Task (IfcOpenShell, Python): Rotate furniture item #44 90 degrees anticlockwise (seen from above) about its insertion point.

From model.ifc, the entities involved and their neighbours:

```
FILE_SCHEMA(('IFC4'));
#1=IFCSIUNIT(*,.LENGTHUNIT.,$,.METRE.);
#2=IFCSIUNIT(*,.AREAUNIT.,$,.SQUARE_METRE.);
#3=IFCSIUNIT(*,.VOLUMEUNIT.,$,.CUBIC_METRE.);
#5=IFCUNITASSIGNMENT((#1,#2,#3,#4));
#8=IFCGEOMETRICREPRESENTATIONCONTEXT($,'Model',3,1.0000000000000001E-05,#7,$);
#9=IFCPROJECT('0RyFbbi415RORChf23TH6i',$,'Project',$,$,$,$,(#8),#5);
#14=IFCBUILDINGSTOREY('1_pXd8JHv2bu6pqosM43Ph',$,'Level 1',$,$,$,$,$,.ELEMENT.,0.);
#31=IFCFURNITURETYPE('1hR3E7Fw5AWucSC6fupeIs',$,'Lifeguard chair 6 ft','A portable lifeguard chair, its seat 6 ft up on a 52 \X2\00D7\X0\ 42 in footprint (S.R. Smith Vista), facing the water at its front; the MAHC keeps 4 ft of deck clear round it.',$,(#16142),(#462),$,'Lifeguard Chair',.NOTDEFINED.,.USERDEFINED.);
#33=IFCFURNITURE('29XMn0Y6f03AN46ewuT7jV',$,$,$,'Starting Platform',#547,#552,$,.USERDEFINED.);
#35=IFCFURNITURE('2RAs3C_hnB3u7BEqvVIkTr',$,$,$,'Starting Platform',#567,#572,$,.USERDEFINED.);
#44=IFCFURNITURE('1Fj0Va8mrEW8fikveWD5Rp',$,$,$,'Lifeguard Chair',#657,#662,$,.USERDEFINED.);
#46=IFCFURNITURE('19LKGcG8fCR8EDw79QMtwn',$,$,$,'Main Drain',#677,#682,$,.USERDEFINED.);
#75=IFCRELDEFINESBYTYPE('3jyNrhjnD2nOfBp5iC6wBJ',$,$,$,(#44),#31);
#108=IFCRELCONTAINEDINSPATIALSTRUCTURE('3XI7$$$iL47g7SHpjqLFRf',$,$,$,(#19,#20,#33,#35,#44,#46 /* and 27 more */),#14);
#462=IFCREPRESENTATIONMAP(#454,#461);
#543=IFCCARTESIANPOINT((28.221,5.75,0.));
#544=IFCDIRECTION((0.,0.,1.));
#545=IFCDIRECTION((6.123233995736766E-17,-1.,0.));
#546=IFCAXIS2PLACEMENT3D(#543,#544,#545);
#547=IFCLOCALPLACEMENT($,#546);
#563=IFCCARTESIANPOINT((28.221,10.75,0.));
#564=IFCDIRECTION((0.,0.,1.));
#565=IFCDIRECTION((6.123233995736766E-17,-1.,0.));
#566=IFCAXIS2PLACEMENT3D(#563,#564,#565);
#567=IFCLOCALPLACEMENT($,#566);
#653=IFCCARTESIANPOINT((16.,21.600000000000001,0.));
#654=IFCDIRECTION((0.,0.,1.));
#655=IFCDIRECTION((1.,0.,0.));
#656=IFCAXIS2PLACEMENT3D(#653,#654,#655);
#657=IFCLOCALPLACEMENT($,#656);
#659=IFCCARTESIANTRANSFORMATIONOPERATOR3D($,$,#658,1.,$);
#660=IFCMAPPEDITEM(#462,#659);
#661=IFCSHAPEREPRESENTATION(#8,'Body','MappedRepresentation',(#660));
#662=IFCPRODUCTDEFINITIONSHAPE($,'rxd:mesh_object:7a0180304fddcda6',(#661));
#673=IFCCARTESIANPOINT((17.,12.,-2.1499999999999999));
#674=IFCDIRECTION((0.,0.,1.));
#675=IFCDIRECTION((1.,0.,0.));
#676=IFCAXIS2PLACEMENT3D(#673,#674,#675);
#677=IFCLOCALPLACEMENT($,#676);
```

```python
import ifcopenshell
import ifcopenshell.api.geometry
import ifcopenshell.util.placement

model = ifcopenshell.open("model.ifc")

item = model.by_guid("1Fj0Va8mrEW8fikveWD5Rp")
matrix = ifcopenshell.util.placement.get_local_placement(item.ObjectPlacement)
matrix = matrix @ ifcopenshell.util.placement.rotation(90, "Z")
ifcopenshell.api.geometry.edit_object_placement(model, product=item, matrix=matrix, is_si=False)

print(ifcopenshell.util.placement.get_local_placement(item.ObjectPlacement).round(3) + 0.0)

model.write("model_v2.ifc")
```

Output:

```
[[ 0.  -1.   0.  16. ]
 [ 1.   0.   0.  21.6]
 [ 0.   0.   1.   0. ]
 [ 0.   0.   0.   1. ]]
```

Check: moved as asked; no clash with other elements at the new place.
